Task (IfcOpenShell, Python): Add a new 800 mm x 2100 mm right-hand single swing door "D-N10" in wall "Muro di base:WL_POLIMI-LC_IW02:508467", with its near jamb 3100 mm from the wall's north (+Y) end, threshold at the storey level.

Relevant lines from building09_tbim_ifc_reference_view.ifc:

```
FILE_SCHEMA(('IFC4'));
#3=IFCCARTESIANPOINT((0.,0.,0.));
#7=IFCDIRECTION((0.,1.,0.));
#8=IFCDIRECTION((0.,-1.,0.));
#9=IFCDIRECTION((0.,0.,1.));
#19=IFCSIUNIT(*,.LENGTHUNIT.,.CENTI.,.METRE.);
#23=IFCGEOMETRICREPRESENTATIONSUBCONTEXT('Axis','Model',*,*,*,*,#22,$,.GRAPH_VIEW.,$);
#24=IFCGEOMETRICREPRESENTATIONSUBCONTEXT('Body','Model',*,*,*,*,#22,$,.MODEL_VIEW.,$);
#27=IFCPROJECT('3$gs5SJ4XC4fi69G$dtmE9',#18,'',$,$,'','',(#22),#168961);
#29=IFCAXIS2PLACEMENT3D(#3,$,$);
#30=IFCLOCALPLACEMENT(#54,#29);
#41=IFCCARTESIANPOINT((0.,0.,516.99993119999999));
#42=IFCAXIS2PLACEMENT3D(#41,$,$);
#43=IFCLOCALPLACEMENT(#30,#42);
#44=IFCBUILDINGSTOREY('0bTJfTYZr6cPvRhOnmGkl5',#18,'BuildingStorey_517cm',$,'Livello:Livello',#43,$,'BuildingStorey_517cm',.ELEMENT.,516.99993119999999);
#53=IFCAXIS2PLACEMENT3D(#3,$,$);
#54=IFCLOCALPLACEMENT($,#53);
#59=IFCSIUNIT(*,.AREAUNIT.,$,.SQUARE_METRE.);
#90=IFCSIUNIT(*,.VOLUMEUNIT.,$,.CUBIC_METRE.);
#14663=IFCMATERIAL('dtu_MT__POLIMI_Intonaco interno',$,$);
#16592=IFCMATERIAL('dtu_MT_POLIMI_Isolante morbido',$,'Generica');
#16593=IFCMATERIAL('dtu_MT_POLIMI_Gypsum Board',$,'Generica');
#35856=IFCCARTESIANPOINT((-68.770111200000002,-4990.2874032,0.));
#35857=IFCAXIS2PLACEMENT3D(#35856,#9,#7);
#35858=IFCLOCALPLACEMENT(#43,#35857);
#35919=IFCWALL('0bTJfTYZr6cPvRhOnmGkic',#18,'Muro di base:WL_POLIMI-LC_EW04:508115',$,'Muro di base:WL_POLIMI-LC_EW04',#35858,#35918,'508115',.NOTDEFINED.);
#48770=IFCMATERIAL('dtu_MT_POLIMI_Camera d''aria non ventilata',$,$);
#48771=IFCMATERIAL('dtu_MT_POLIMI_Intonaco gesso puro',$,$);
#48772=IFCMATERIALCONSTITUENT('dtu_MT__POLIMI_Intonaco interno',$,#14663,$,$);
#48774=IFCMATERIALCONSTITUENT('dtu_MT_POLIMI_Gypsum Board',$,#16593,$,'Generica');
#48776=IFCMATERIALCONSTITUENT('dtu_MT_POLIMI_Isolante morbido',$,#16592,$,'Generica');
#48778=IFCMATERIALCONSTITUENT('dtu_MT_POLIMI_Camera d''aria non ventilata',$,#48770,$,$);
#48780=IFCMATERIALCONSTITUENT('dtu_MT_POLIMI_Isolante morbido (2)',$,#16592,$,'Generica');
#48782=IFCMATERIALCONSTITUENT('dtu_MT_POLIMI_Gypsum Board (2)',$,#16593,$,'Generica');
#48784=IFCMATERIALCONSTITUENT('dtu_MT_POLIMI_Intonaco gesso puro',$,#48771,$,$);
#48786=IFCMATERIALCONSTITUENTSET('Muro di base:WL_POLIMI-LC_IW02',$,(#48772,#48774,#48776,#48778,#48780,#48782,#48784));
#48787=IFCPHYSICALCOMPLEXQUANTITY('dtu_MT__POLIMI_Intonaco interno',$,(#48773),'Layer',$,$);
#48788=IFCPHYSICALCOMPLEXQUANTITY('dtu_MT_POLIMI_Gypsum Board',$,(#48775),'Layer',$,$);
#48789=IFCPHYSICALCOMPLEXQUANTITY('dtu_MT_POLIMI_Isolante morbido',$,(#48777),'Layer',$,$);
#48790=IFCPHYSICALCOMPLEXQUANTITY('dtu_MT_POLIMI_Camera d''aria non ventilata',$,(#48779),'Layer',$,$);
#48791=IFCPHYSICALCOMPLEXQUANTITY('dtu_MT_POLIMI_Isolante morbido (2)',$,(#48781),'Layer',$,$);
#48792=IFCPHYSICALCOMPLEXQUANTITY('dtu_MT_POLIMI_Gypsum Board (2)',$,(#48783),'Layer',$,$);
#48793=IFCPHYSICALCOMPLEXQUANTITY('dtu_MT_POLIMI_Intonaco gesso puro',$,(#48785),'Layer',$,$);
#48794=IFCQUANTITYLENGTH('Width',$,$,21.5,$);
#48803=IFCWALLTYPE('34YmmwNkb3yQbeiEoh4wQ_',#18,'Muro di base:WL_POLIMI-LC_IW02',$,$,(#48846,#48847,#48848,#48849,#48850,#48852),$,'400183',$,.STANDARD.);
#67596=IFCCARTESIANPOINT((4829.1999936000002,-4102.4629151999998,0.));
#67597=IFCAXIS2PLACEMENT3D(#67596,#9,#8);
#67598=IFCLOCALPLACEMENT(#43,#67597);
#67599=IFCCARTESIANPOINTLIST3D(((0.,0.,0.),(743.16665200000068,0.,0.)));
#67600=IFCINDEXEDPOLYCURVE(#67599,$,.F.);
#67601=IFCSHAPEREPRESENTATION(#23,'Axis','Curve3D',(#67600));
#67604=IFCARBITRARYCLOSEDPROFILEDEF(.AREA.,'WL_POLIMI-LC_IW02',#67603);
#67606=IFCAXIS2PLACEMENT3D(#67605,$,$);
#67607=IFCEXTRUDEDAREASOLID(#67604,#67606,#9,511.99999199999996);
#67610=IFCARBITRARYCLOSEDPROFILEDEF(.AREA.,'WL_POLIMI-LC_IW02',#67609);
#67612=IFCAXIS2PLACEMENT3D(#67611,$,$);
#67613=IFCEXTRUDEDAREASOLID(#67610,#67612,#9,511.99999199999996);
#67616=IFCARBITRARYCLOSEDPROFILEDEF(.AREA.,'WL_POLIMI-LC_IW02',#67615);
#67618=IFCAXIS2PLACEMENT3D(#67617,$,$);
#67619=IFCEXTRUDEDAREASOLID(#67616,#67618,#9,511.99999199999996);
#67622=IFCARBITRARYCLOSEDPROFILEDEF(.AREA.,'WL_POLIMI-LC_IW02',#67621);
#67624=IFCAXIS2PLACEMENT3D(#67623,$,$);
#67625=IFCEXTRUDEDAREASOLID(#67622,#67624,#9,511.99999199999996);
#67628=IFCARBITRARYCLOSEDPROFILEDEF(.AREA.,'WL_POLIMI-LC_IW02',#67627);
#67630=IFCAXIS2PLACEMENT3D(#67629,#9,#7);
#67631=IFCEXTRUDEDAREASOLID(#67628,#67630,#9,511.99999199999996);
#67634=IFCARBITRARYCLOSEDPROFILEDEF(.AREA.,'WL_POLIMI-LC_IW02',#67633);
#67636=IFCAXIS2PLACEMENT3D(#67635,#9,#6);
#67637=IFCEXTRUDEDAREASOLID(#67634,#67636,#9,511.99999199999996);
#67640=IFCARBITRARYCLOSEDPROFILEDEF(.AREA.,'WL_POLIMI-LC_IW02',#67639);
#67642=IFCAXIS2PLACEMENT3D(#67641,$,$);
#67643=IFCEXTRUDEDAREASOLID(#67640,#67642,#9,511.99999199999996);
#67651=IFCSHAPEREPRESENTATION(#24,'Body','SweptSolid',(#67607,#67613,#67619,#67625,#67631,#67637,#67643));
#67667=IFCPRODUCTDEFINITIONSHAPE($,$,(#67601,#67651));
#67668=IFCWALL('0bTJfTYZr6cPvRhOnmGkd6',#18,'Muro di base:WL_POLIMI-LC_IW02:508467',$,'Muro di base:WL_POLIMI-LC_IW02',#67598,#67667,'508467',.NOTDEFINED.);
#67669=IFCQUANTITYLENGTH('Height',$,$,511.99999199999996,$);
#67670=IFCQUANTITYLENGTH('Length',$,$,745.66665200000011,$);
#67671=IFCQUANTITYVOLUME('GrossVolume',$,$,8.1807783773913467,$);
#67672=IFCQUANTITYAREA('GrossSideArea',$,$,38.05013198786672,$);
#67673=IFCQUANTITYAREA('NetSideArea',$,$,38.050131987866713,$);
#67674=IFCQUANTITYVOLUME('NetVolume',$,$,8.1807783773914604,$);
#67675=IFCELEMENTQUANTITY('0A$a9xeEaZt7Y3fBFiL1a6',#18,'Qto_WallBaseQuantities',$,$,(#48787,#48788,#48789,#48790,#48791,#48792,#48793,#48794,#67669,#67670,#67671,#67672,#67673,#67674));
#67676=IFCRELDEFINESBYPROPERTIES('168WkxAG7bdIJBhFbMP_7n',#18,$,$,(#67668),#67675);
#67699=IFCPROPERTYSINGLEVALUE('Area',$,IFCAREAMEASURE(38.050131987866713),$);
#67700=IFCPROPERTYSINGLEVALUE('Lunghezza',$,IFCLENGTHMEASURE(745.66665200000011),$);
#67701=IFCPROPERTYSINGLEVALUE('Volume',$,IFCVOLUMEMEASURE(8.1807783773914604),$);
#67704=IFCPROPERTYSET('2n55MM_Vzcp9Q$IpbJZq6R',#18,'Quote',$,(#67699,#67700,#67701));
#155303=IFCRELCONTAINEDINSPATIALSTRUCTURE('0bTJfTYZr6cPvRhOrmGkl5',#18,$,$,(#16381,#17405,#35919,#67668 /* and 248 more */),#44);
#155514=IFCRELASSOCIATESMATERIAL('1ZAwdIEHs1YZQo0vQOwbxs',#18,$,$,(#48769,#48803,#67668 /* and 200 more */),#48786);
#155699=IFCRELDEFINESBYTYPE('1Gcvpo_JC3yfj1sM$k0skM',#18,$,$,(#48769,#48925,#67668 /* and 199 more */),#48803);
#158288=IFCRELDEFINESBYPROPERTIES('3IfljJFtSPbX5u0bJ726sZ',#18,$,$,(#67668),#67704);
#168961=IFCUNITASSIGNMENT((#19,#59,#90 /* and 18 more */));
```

```python
import numpy as np
import ifcopenshell
import ifcopenshell.api.feature
import ifcopenshell.api.geometry
import ifcopenshell.api.pset
import ifcopenshell.api.root
import ifcopenshell.api.spatial
import ifcopenshell.geom
import ifcopenshell.util.element
import ifcopenshell.util.placement
import ifcopenshell.util.representation
import ifcopenshell.util.shape
import ifcopenshell.util.unit

model = ifcopenshell.open("building09_tbim_ifc_reference_view.ifc")
unit_scale = ifcopenshell.util.unit.calculate_unit_scale(model)
area_scale = ifcopenshell.util.unit.calculate_unit_scale(model, "AREAUNIT")
volume_scale = ifcopenshell.util.unit.calculate_unit_scale(model, "VOLUMEUNIT")
settings = ifcopenshell.geom.settings()


def volume(element):
    """Net volume in cubic metres, openings subtracted."""
    shape = ifcopenshell.geom.create_shape(settings, element)
    return ifcopenshell.util.shape.get_volume(shape.geometry)


wall = model.by_guid("0bTJfTYZr6cPvRhOnmGkd6")
storey = ifcopenshell.util.element.get_container(wall, ifc_class="IfcBuildingStorey")
context = ifcopenshell.util.representation.get_context(model, "Model", "Body", "MODEL_VIEW")
before = volume(wall)

width, height, from_end, sill = 0.8, 2.1, 3.1, 0.0  # metres

# The wall runs along its own X axis, and the end named is its -X end.
wall_shape = ifcopenshell.geom.create_shape(settings, wall)
x, y, z = ifcopenshell.util.shape.get_vertices(wall_shape.geometry).T
start = x.min() + from_end
face, thickness = float(y.min()), float(y.max() - y.min())
wall_matrix = ifcopenshell.util.placement.get_local_placement(wall.ObjectPlacement)
level = ifcopenshell.util.placement.get_local_placement(storey.ObjectPlacement)[2, 3]


def in_wall(x, y):
    """Placement at x, y metres in the wall's axes, at sill height."""
    matrix = wall_matrix.copy()
    matrix[:, 3] = wall_matrix @ np.array([x / unit_scale, y / unit_scale, 0.0, 1.0])
    matrix[2, 3] = level + sill / unit_scale
    return matrix


# Opening: a box that overshoots both wall faces by 50 mm.
opening = ifcopenshell.api.root.create_entity(model, ifc_class="IfcOpeningElement", predefined_type="OPENING")
box = ifcopenshell.api.geometry.add_wall_representation(
    model, context=context, length=width, height=height, thickness=thickness + 0.1
)
ifcopenshell.api.geometry.assign_representation(model, product=opening, representation=box)
ifcopenshell.api.geometry.edit_object_placement(model, product=opening, matrix=in_wall(start, face - 0.05), is_si=False)
ifcopenshell.api.feature.add_feature(model, feature=opening, element=wall)

door = ifcopenshell.api.root.create_entity(model, ifc_class="IfcDoor", name="D-N10", predefined_type="DOOR")
door.OverallWidth, door.OverallHeight = width / unit_scale, height / unit_scale
door.OperationType = "SINGLE_SWING_RIGHT"
body = ifcopenshell.api.geometry.add_door_representation(
    model,
    context=context,
    overall_width=door.OverallWidth,
    overall_height=door.OverallHeight,
    operation_type="SINGLE_SWING_RIGHT",
    lining_properties={"LiningDepth": thickness / unit_scale, "ThresholdDepth": thickness / unit_scale},
)
ifcopenshell.api.geometry.assign_representation(model, product=door, representation=body)
ifcopenshell.api.spatial.assign_container(model, products=[door], relating_structure=storey)
ifcopenshell.api.feature.add_filling(model, opening=opening, element=door)

# The lining spans the wall, so the door starts at the wall face.
ifcopenshell.api.geometry.edit_object_placement(model, product=door, matrix=in_wall(start, face), is_si=False)

after = volume(wall)

# Update the wall's stored quantities.
qto = model.by_id(ifcopenshell.util.element.get_pset(wall, "Qto_WallBaseQuantities", should_inherit=False)["id"])
ifcopenshell.api.pset.edit_qto(model, qto=qto, properties={
    "NetSideArea": after / thickness / area_scale,
    "NetVolume": after / volume_scale,
})
pset = model.by_id(ifcopenshell.util.element.get_pset(wall, "Quote", should_inherit=False)["id"])
ifcopenshell.api.pset.edit_pset(model, pset=pset, properties={
    "Area": model.create_entity("IfcAreaMeasure", after / thickness / area_scale),
    "Volume": model.create_entity("IfcVolumeMeasure", after / volume_scale),
})

print(f"wall volume {before:.3f} -> {after:.3f} m3")

model.write("building09_tbim_ifc_reference_view_v2.ifc")
```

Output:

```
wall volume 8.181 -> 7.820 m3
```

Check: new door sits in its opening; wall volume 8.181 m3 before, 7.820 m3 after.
